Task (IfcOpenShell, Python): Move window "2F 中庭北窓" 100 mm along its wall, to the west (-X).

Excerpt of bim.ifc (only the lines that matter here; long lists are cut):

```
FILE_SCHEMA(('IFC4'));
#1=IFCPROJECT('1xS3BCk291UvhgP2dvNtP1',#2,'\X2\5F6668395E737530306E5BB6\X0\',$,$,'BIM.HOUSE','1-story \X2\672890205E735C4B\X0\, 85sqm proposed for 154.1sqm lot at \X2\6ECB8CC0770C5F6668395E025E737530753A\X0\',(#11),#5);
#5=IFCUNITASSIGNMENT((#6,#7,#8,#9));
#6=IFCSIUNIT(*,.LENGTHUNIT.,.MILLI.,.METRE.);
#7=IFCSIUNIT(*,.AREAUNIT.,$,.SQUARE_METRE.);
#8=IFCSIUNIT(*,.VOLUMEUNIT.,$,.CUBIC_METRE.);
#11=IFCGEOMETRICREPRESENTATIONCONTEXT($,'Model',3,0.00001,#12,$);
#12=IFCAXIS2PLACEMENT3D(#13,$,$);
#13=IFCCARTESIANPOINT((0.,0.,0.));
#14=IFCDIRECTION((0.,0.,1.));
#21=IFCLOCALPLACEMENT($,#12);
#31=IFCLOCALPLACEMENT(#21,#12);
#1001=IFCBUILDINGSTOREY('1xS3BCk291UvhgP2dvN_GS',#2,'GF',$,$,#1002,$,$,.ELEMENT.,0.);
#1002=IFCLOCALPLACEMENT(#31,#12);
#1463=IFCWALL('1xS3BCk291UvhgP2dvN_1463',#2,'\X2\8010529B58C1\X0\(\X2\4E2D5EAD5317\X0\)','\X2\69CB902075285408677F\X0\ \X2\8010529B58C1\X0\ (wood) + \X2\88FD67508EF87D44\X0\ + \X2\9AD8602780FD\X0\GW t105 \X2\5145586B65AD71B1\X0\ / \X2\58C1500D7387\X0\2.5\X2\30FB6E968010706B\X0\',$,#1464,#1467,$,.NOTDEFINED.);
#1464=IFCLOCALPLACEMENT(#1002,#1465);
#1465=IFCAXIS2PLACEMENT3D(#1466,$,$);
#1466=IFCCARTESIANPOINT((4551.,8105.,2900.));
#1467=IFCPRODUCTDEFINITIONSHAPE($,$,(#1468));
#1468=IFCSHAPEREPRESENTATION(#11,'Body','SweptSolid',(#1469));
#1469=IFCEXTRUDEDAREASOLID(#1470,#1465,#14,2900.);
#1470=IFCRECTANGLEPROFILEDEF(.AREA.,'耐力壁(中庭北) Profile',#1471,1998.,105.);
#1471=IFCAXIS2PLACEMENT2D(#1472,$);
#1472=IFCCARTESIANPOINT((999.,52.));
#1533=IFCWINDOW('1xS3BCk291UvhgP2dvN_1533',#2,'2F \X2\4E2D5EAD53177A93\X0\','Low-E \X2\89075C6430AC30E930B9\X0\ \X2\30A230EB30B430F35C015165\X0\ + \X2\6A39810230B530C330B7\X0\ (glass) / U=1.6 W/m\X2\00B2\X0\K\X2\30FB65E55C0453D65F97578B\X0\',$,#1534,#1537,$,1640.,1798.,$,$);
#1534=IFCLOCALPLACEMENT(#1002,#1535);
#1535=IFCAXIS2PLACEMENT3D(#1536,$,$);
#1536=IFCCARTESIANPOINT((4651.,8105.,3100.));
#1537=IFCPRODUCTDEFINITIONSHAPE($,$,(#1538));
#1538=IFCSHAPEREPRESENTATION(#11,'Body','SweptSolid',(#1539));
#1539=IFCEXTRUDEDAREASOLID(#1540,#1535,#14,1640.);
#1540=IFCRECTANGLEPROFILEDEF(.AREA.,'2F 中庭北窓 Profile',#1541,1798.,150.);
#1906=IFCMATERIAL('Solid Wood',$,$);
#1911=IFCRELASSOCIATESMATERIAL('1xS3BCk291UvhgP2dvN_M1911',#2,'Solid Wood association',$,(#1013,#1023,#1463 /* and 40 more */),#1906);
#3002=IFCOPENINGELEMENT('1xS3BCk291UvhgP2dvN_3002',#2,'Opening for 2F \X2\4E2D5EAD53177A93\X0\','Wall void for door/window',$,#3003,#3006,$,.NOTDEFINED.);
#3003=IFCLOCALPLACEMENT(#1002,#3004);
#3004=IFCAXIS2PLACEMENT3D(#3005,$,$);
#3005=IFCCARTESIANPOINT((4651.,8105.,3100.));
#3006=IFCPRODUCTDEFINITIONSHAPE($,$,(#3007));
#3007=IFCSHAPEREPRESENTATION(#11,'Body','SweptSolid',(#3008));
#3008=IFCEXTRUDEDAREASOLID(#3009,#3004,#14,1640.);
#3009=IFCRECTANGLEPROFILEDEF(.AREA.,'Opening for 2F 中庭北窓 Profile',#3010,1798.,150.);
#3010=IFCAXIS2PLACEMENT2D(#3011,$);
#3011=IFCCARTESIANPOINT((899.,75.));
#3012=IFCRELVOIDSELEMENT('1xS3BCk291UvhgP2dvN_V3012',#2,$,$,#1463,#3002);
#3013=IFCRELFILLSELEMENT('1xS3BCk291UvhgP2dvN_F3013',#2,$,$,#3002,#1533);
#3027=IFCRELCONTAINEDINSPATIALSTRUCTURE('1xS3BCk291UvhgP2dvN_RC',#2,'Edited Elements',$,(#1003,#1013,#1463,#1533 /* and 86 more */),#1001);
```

```python
import ifcopenshell
import ifcopenshell.api.geometry
import ifcopenshell.util.placement

model = ifcopenshell.open("bim.ifc")

window = model.by_guid("1xS3BCk291UvhgP2dvN_1533")
opening = window.FillsVoids[0].RelatingOpeningElement
wall = opening.VoidsElements[0].RelatingBuildingElement

wall_matrix = ifcopenshell.util.placement.get_local_placement(wall.ObjectPlacement)
shift = wall_matrix[:3, 0] * -100.0
before = ifcopenshell.util.placement.get_local_placement(window.ObjectPlacement)[:3, 3].copy()

# The window is not placed relative to its opening, so move both.
for product in (opening, window):
    matrix = ifcopenshell.util.placement.get_local_placement(product.ObjectPlacement)
    matrix[:3, 3] += shift
    ifcopenshell.api.geometry.edit_object_placement(model, product=product, matrix=matrix, is_si=False)

after = ifcopenshell.util.placement.get_local_placement(window.ObjectPlacement)[:3, 3]
print("window moved by", (after - before).round(3) + 0.0)

model.write("bim_updated.ifc")
```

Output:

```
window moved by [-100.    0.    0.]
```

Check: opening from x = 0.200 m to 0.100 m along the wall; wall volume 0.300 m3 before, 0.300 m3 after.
